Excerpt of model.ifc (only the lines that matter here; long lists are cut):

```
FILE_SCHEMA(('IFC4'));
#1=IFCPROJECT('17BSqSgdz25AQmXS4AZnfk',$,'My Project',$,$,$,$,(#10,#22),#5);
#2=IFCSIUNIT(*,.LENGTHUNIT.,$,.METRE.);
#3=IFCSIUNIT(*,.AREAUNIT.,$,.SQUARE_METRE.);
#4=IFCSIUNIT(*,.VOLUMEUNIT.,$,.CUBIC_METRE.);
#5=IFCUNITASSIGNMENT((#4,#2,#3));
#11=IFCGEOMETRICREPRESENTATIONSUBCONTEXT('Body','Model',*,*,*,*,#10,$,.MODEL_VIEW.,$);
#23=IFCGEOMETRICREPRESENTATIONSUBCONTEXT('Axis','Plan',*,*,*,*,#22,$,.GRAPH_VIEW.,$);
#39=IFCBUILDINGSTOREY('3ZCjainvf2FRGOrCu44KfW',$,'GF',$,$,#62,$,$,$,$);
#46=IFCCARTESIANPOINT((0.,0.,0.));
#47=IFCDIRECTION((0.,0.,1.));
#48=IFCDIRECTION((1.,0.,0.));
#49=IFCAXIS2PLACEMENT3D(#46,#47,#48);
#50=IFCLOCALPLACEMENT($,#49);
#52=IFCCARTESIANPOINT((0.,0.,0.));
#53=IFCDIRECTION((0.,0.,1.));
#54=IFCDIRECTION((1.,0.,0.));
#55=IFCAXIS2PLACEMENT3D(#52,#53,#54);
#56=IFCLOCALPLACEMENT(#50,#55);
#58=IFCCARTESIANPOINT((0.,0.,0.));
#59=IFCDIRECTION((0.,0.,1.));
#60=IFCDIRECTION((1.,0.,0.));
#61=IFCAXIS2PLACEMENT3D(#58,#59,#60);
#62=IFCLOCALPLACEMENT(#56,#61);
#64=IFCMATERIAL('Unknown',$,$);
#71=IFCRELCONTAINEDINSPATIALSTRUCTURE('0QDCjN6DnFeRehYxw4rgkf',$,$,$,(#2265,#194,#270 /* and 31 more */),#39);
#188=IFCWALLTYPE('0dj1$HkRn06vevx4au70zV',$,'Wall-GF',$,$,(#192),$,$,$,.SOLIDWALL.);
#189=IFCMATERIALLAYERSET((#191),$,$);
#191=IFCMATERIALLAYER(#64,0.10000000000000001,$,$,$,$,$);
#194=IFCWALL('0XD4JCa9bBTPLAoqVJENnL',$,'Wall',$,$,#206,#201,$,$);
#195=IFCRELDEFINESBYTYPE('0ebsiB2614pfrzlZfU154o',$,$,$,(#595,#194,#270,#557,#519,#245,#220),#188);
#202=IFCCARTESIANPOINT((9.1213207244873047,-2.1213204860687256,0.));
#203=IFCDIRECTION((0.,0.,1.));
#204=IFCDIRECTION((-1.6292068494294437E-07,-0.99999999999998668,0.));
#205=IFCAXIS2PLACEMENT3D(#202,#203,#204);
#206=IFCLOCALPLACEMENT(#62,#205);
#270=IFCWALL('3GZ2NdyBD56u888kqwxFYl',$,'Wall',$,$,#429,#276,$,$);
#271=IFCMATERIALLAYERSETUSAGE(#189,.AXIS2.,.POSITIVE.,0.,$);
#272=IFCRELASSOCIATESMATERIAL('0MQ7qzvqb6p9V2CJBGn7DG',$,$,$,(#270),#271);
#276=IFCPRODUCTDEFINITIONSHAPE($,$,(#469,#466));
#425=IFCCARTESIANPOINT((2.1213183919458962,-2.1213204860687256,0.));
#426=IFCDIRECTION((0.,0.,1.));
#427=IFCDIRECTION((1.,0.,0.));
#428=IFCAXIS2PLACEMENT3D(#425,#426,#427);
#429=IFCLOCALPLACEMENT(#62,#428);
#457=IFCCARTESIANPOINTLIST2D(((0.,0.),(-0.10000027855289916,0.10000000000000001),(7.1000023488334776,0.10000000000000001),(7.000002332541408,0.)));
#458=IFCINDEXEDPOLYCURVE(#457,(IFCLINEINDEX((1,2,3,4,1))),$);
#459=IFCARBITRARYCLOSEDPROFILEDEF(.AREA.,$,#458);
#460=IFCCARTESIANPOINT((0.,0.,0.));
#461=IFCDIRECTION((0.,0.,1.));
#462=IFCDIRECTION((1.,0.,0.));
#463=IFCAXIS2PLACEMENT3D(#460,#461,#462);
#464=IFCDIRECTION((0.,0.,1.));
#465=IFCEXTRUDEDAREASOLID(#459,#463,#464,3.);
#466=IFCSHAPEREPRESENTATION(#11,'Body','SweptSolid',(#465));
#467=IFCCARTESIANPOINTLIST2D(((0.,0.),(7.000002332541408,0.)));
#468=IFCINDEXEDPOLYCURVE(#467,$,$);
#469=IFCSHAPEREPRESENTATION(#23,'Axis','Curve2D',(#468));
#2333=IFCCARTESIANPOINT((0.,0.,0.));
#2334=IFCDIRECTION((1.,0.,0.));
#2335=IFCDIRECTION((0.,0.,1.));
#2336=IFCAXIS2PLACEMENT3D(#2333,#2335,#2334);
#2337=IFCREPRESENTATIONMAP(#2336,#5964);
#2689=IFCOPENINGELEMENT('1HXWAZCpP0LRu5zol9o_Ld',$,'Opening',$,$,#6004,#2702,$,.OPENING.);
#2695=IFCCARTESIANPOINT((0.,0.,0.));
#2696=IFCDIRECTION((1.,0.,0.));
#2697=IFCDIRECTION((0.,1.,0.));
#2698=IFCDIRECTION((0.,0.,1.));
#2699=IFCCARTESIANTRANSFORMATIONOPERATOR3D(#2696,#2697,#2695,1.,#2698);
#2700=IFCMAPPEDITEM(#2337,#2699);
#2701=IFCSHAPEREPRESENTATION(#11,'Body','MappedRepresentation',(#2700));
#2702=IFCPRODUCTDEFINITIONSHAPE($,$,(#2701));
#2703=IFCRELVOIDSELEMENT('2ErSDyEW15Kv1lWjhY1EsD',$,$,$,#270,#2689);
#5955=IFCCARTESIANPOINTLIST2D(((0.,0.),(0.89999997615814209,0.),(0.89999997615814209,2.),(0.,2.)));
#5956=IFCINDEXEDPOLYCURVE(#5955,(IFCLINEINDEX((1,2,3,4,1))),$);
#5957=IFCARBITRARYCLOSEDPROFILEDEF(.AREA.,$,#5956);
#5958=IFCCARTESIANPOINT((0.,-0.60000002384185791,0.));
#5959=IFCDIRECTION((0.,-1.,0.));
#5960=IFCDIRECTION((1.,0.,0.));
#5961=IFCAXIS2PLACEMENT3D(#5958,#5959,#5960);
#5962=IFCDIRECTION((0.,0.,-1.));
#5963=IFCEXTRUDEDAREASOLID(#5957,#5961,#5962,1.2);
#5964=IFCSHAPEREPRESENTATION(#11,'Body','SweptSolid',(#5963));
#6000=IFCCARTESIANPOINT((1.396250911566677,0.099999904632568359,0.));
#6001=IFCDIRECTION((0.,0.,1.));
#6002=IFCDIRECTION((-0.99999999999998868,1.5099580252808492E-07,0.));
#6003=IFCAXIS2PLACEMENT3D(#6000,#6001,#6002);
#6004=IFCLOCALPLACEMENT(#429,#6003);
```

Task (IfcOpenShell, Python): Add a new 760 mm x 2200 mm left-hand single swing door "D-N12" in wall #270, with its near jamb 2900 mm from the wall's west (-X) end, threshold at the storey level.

```python
import numpy as np
import ifcopenshell
import ifcopenshell.api.feature
import ifcopenshell.api.geometry
import ifcopenshell.api.root
import ifcopenshell.api.spatial
import ifcopenshell.geom
import ifcopenshell.util.element
import ifcopenshell.util.placement
import ifcopenshell.util.representation
import ifcopenshell.util.shape
import ifcopenshell.util.unit

model = ifcopenshell.open("model.ifc")
unit_scale = ifcopenshell.util.unit.calculate_unit_scale(model)
settings = ifcopenshell.geom.settings()


def volume(element):
    """Net volume in cubic metres, openings subtracted."""
    shape = ifcopenshell.geom.create_shape(settings, element)
    return ifcopenshell.util.shape.get_volume(shape.geometry)


wall = model.by_guid("3GZ2NdyBD56u888kqwxFYl")
storey = ifcopenshell.util.element.get_container(wall, ifc_class="IfcBuildingStorey")
context = ifcopenshell.util.representation.get_context(model, "Model", "Body", "MODEL_VIEW")
before = volume(wall)

width, height, from_end, sill = 0.76, 2.2, 2.9, 0.0  # metres

# The wall runs along its own X axis, and the end named is its -X end.
wall_shape = ifcopenshell.geom.create_shape(settings, wall)
x, y, z = ifcopenshell.util.shape.get_vertices(wall_shape.geometry).T
start = x.min() + from_end
face, thickness = float(y.min()), float(y.max() - y.min())
wall_matrix = ifcopenshell.util.placement.get_local_placement(wall.ObjectPlacement)
level = ifcopenshell.util.placement.get_local_placement(storey.ObjectPlacement)[2, 3]


def in_wall(x, y):
    """Placement at x, y metres in the wall's axes, at sill height."""
    matrix = wall_matrix.copy()
    matrix[:, 3] = wall_matrix @ np.array([x / unit_scale, y / unit_scale, 0.0, 1.0])
    matrix[2, 3] = level + sill / unit_scale
    return matrix


# Opening: a box that overshoots both wall faces by 50 mm.
opening = ifcopenshell.api.root.create_entity(model, ifc_class="IfcOpeningElement", predefined_type="OPENING")
box = ifcopenshell.api.geometry.add_wall_representation(
    model, context=context, length=width, height=height, thickness=thickness + 0.1
)
ifcopenshell.api.geometry.assign_representation(model, product=opening, representation=box)
ifcopenshell.api.geometry.edit_object_placement(model, product=opening, matrix=in_wall(start, face - 0.05), is_si=False)
ifcopenshell.api.feature.add_feature(model, feature=opening, element=wall)

door = ifcopenshell.api.root.create_entity(model, ifc_class="IfcDoor", name="D-N12", predefined_type="DOOR")
door.OverallWidth, door.OverallHeight = width / unit_scale, height / unit_scale
door.OperationType = "SINGLE_SWING_LEFT"
body = ifcopenshell.api.geometry.add_door_representation(
    model,
    context=context,
    overall_width=door.OverallWidth,
    overall_height=door.OverallHeight,
    operation_type="SINGLE_SWING_LEFT",
    lining_properties={"LiningDepth": thickness / unit_scale, "ThresholdDepth": thickness / unit_scale},
)
ifcopenshell.api.geometry.assign_representation(model, product=door, representation=body)
ifcopenshell.api.spatial.assign_container(model, products=[door], relating_structure=storey)
ifcopenshell.api.feature.add_filling(model, opening=opening, element=door)

# The lining spans the wall, so the door starts at the wall face.
ifcopenshell.api.geometry.edit_object_placement(model, product=door, matrix=in_wall(start, face), is_si=False)

after = volume(wall)

print(f"wall volume {before:.3f} -> {after:.3f} m3")

model.write("model-out.ifc")
```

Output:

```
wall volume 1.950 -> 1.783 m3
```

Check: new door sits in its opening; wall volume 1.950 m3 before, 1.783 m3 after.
